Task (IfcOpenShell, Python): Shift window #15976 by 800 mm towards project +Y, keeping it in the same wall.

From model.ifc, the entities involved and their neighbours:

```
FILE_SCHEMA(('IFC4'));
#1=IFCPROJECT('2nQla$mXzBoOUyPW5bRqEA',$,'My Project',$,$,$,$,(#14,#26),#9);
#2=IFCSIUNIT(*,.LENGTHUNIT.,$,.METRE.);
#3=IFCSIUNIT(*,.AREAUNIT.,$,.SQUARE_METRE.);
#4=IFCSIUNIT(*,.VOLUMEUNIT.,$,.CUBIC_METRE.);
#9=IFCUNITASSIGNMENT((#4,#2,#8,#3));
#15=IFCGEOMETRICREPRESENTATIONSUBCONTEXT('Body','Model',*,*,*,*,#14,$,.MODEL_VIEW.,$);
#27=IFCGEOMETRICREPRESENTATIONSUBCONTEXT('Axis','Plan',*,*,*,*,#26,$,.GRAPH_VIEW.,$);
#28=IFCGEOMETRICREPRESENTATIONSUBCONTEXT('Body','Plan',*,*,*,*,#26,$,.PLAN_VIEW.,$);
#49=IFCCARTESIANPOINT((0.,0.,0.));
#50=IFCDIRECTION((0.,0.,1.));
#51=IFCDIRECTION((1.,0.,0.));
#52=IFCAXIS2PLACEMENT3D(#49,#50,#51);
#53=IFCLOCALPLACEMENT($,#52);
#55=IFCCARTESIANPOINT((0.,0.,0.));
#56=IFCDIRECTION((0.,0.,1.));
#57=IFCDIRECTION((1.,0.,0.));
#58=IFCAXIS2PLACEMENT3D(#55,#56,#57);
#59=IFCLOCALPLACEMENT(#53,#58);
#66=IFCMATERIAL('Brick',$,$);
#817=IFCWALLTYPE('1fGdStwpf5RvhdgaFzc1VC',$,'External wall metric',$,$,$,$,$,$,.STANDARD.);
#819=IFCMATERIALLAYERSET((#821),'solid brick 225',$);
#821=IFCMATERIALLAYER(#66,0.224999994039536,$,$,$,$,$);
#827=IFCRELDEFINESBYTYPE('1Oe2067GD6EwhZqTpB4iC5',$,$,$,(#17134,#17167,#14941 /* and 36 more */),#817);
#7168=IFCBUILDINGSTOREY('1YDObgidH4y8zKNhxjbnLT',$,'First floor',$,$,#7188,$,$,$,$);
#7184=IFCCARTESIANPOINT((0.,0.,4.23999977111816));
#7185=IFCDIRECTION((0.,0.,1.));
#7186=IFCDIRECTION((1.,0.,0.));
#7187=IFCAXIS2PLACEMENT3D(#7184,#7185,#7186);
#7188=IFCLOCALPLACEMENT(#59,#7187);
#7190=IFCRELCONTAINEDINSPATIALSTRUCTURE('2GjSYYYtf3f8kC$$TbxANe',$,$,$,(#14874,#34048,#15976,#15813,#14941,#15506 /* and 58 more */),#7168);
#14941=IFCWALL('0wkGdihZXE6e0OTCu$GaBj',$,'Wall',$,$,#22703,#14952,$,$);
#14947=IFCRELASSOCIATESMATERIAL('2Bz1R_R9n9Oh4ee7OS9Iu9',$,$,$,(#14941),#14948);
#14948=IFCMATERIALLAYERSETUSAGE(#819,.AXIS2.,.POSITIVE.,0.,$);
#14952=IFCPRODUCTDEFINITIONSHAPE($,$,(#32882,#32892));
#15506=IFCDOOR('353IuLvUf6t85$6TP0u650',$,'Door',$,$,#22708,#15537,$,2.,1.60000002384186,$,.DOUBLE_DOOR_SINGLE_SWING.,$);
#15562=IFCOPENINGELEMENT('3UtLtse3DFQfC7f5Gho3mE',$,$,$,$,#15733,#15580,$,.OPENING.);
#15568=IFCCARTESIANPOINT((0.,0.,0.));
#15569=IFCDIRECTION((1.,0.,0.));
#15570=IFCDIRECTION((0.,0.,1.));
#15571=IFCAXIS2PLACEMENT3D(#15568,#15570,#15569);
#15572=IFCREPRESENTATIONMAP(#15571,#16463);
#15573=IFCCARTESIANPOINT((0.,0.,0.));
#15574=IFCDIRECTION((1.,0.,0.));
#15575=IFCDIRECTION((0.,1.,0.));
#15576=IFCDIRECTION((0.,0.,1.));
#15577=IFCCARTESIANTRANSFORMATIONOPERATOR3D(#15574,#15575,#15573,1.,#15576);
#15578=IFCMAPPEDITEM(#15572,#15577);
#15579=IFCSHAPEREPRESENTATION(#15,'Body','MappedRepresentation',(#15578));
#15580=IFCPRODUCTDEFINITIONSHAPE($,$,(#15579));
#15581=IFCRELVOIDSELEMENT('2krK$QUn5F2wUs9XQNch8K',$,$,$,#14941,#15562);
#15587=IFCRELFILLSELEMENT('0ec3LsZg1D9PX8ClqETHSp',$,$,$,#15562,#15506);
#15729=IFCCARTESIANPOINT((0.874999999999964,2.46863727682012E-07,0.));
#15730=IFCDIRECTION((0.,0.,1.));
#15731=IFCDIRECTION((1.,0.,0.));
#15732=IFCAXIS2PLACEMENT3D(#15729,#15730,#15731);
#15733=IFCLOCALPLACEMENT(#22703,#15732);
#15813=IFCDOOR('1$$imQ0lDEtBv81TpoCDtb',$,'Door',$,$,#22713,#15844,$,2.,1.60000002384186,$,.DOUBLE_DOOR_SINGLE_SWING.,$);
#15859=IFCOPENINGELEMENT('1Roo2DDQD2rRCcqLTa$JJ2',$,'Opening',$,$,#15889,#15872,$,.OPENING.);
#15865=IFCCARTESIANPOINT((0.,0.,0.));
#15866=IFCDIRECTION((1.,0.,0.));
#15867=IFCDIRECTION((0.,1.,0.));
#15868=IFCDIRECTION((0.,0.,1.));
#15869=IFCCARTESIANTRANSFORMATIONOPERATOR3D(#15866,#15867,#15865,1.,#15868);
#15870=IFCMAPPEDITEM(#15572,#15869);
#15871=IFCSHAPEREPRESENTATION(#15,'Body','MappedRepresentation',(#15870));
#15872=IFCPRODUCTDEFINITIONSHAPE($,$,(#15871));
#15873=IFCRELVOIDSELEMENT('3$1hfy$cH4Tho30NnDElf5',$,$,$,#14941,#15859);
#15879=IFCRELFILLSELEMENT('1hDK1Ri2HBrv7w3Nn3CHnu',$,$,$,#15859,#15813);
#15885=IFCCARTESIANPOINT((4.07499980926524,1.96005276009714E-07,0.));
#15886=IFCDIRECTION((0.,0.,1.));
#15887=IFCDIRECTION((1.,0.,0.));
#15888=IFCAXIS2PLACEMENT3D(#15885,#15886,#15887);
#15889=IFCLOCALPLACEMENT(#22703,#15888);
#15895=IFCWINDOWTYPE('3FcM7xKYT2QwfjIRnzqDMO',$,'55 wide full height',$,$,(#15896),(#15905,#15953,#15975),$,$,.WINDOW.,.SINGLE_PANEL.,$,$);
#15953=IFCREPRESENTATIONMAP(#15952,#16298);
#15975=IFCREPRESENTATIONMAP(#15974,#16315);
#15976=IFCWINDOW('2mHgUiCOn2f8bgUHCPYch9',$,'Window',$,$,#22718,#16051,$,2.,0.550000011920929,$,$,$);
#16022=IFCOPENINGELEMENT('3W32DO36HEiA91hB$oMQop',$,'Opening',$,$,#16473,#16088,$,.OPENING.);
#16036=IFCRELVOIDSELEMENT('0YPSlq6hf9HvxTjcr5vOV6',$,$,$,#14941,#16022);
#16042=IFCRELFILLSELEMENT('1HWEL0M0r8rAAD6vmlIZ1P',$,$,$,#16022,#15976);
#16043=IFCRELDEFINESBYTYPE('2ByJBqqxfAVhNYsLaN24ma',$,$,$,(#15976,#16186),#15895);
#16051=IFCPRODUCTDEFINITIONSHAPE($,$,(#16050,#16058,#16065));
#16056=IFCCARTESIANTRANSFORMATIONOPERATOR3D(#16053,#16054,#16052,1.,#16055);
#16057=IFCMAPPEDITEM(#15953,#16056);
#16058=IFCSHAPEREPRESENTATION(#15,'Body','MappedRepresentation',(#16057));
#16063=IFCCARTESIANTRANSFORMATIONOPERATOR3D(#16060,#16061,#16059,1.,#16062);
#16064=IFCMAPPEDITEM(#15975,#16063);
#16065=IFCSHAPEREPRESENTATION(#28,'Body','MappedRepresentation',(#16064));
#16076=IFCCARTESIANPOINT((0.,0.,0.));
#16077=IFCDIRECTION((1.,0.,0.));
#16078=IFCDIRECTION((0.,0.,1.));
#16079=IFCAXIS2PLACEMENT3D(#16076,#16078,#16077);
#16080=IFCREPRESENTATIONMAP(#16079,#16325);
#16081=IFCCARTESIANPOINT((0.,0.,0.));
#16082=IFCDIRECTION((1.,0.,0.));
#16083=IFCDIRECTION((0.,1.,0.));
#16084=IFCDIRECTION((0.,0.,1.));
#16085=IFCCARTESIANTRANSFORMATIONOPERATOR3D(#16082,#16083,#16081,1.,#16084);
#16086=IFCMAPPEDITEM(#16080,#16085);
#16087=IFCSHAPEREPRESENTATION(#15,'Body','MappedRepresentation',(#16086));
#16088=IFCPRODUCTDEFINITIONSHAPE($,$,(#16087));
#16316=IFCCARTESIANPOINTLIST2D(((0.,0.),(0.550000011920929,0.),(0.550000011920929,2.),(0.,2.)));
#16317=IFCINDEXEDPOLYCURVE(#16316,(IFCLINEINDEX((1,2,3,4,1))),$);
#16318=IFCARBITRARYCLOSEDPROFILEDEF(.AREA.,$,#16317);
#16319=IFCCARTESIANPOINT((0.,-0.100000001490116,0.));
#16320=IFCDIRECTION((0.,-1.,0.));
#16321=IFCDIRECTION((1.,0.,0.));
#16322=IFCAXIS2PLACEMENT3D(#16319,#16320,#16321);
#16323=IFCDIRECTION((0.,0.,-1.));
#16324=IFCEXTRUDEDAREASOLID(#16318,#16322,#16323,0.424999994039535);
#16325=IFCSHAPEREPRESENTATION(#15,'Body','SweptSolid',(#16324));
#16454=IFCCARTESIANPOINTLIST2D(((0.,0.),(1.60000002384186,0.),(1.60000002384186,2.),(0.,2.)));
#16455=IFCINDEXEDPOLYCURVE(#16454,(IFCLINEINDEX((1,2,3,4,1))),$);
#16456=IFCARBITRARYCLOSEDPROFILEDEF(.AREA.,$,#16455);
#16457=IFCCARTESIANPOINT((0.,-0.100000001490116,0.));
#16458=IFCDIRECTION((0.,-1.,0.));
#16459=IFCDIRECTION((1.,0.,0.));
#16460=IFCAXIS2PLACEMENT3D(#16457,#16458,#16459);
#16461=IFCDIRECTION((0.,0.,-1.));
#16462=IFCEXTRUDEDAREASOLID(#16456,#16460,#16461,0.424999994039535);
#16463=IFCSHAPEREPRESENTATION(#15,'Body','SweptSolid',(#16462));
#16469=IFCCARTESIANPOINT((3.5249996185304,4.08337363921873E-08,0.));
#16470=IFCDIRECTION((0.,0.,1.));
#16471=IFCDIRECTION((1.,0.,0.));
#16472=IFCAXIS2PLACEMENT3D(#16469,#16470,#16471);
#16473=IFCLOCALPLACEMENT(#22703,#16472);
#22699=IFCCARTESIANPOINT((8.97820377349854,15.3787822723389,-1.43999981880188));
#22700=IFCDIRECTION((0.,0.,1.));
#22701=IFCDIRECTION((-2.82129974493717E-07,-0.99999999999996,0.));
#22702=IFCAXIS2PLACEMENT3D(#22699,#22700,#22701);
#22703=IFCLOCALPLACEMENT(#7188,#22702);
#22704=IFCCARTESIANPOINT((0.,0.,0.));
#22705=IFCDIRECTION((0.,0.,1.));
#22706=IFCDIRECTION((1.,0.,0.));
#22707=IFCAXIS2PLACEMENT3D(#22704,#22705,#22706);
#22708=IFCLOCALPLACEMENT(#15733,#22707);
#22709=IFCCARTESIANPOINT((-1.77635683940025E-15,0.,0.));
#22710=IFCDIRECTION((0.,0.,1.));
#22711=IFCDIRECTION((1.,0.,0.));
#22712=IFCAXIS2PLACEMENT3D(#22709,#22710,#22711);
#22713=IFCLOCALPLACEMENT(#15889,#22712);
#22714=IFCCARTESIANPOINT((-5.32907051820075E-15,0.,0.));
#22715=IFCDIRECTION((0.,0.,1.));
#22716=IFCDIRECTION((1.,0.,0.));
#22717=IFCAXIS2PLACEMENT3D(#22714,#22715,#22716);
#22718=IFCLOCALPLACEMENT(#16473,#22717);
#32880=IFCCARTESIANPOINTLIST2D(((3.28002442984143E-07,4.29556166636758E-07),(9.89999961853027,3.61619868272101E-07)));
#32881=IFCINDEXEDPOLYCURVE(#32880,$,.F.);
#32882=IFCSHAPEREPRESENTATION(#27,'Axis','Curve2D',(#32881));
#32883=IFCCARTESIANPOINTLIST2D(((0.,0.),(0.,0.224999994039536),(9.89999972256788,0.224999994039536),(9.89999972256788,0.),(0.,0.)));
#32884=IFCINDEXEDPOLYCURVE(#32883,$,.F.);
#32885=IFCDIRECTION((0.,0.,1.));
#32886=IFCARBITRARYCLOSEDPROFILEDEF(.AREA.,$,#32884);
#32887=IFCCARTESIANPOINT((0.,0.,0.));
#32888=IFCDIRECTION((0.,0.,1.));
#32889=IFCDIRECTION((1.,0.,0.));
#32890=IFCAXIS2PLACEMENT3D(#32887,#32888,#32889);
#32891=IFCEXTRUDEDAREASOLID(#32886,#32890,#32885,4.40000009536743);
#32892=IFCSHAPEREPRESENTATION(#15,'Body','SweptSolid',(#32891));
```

```python
import ifcopenshell
import ifcopenshell.api.geometry
import ifcopenshell.util.placement

model = ifcopenshell.open("model.ifc")

window = model.by_guid("2mHgUiCOn2f8bgUHCPYch9")
opening = window.FillsVoids[0].RelatingOpeningElement
wall = opening.VoidsElements[0].RelatingBuildingElement

wall_matrix = ifcopenshell.util.placement.get_local_placement(wall.ObjectPlacement)
shift = wall_matrix[:3, 0] * -0.8
before = ifcopenshell.util.placement.get_local_placement(window.ObjectPlacement)[:3, 3].copy()

# The window is placed relative to its opening, so it follows when the opening moves.
matrix = ifcopenshell.util.placement.get_local_placement(opening.ObjectPlacement)
matrix[:3, 3] += shift
ifcopenshell.api.geometry.edit_object_placement(
    model, product=opening, matrix=matrix, is_si=False, should_transform_children=True
)

after = ifcopenshell.util.placement.get_local_placement(window.ObjectPlacement)[:3, 3]
print("window moved by", (after - before).round(3) + 0.0)

model.write("model_updated.ifc")
```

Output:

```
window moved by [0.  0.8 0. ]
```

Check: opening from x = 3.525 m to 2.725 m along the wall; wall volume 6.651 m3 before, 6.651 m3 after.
